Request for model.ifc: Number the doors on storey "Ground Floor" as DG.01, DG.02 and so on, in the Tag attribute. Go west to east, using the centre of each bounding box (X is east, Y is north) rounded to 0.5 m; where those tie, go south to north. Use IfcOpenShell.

First a look at what the model holds.

```python
import ifcopenshell
import ifcopenshell.util.element
import ifcopenshell.util.placement

model = ifcopenshell.open("model.ifc")
print(model.schema)
storey = next(s for s in model.by_type("IfcBuildingStorey") if s.Name == "Ground Floor")
doors = [e for e in ifcopenshell.util.element.get_decomposition(storey) if e.is_a("IfcDoor")]
for e in sorted(doors, key=lambda e: e.id()):
    origin = ifcopenshell.util.placement.get_local_placement(e.ObjectPlacement)[:3, 3]
    print(e.id(), e.Tag, e.Name, origin.round(2) + 0.0, sep=" | ")
```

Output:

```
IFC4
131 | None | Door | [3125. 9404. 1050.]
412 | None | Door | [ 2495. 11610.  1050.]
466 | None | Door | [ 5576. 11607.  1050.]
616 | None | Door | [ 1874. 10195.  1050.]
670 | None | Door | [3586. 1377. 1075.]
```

```python
import ifcopenshell
import ifcopenshell.geom
import ifcopenshell.util.element
import ifcopenshell.util.shape

model = ifcopenshell.open("model.ifc")
settings = ifcopenshell.geom.settings()
settings.set("use-world-coords", True)


def centre(element):
    shape = ifcopenshell.geom.create_shape(settings, element)
    return ifcopenshell.util.shape.get_bbox_centroid(shape.geometry)


storey = next(s for s in model.by_type("IfcBuildingStorey") if s.Name == "Ground Floor")
doors = [e for e in ifcopenshell.util.element.get_decomposition(storey) if e.is_a("IfcDoor")]

# Insertion points can sit at a corner or the storey origin, so sort by the geometry (in metres).
centres = {e: centre(e) for e in doors}
doors.sort(key=lambda e: (round(centres[e][0] / 0.5), centres[e][1]))

for i, e in enumerate(doors, start=1):
    number = f"DG.{i:02d}"
    e.Tag = number
    print(e.id(), number)

model.write("model_rev.ifc")
```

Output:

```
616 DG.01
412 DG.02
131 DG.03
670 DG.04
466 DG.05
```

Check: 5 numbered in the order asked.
